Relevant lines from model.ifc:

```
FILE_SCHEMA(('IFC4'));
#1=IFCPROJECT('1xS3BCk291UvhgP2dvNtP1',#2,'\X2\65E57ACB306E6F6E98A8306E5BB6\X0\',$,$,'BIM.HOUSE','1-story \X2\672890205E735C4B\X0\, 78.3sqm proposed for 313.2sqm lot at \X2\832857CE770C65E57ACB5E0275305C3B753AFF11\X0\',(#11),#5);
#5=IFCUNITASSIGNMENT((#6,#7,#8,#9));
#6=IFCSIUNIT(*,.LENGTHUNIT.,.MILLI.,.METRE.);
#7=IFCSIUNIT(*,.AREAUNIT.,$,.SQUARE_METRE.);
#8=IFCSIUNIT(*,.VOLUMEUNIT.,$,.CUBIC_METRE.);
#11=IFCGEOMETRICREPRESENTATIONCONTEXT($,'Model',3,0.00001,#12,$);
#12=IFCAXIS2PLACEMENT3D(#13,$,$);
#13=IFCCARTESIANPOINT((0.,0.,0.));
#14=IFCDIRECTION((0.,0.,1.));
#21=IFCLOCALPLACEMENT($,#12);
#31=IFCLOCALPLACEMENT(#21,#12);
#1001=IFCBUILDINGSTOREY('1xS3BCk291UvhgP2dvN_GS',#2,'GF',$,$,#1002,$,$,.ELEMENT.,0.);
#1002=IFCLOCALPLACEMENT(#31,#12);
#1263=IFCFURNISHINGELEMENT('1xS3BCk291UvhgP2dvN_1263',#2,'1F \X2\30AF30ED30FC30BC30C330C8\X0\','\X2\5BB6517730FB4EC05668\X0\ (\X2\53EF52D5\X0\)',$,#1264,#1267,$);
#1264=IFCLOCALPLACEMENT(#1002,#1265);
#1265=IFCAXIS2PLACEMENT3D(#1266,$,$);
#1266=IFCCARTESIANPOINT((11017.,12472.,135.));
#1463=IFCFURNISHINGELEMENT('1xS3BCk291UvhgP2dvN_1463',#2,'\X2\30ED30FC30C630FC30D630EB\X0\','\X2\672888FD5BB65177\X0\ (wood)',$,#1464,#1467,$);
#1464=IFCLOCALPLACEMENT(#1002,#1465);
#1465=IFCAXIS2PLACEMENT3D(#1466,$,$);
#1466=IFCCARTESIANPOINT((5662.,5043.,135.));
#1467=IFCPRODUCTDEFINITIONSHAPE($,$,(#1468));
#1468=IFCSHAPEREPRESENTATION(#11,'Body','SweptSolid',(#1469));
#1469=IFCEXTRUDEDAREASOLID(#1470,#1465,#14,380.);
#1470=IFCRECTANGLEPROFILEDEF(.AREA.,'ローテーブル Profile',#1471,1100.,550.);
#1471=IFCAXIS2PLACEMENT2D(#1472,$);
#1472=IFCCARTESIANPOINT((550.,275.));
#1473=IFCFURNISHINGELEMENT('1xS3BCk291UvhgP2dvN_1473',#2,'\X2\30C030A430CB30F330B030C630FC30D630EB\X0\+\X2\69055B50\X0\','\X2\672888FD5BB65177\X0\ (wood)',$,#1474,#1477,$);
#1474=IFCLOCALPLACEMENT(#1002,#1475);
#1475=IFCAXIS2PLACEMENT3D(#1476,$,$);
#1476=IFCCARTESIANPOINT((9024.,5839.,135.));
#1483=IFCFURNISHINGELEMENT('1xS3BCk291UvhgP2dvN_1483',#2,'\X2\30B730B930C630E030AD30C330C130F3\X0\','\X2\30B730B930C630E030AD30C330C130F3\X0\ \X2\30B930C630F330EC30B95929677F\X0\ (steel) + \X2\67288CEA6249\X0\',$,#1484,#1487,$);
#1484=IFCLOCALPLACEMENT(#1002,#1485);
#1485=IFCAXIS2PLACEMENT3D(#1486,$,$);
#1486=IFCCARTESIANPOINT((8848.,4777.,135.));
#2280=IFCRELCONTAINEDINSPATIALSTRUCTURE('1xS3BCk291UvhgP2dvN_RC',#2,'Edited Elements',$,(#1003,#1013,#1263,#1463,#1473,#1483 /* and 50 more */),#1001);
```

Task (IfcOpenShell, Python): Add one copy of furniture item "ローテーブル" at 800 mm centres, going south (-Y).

```python
import numpy as np
import ifcopenshell
import ifcopenshell.api.geometry
import ifcopenshell.api.root
import ifcopenshell.util.element
import ifcopenshell.util.placement

model = ifcopenshell.open("model.ifc")


def reuse_history(source, copy):
    """copy_class also copies each property set's owner history, people and application; keep the originals."""
    for rel in copy.IsDefinedBy:
        if rel.is_a("IfcRelDefinesByProperties") and (history := rel.RelatingPropertyDefinition.OwnerHistory):
            rel.RelatingPropertyDefinition.OwnerHistory = source.OwnerHistory
            ifcopenshell.util.element.remove_deep2(model, history)


source = model.by_id(1463)
base = ifcopenshell.util.placement.get_local_placement(source.ObjectPlacement)
step = np.array([0.0, -1.0, 0.0]) * 800.0

for i in range(1, 2):
    copy = ifcopenshell.api.root.copy_class(model, product=source)
    copy.Representation = ifcopenshell.util.element.copy_deep(
        model, source.Representation, exclude=["IfcGeometricRepresentationContext", "IfcRepresentationMap"]
    )
    reuse_history(source, copy)
    matrix = base.copy()
    matrix[:3, 3] += i * step
    print("added at", matrix[:3, 3].round(3) + 0.0)
    ifcopenshell.api.geometry.edit_object_placement(model, product=copy, matrix=matrix, is_si=False)

model.write("model_edited.ifc")
```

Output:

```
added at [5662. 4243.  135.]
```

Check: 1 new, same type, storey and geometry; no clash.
